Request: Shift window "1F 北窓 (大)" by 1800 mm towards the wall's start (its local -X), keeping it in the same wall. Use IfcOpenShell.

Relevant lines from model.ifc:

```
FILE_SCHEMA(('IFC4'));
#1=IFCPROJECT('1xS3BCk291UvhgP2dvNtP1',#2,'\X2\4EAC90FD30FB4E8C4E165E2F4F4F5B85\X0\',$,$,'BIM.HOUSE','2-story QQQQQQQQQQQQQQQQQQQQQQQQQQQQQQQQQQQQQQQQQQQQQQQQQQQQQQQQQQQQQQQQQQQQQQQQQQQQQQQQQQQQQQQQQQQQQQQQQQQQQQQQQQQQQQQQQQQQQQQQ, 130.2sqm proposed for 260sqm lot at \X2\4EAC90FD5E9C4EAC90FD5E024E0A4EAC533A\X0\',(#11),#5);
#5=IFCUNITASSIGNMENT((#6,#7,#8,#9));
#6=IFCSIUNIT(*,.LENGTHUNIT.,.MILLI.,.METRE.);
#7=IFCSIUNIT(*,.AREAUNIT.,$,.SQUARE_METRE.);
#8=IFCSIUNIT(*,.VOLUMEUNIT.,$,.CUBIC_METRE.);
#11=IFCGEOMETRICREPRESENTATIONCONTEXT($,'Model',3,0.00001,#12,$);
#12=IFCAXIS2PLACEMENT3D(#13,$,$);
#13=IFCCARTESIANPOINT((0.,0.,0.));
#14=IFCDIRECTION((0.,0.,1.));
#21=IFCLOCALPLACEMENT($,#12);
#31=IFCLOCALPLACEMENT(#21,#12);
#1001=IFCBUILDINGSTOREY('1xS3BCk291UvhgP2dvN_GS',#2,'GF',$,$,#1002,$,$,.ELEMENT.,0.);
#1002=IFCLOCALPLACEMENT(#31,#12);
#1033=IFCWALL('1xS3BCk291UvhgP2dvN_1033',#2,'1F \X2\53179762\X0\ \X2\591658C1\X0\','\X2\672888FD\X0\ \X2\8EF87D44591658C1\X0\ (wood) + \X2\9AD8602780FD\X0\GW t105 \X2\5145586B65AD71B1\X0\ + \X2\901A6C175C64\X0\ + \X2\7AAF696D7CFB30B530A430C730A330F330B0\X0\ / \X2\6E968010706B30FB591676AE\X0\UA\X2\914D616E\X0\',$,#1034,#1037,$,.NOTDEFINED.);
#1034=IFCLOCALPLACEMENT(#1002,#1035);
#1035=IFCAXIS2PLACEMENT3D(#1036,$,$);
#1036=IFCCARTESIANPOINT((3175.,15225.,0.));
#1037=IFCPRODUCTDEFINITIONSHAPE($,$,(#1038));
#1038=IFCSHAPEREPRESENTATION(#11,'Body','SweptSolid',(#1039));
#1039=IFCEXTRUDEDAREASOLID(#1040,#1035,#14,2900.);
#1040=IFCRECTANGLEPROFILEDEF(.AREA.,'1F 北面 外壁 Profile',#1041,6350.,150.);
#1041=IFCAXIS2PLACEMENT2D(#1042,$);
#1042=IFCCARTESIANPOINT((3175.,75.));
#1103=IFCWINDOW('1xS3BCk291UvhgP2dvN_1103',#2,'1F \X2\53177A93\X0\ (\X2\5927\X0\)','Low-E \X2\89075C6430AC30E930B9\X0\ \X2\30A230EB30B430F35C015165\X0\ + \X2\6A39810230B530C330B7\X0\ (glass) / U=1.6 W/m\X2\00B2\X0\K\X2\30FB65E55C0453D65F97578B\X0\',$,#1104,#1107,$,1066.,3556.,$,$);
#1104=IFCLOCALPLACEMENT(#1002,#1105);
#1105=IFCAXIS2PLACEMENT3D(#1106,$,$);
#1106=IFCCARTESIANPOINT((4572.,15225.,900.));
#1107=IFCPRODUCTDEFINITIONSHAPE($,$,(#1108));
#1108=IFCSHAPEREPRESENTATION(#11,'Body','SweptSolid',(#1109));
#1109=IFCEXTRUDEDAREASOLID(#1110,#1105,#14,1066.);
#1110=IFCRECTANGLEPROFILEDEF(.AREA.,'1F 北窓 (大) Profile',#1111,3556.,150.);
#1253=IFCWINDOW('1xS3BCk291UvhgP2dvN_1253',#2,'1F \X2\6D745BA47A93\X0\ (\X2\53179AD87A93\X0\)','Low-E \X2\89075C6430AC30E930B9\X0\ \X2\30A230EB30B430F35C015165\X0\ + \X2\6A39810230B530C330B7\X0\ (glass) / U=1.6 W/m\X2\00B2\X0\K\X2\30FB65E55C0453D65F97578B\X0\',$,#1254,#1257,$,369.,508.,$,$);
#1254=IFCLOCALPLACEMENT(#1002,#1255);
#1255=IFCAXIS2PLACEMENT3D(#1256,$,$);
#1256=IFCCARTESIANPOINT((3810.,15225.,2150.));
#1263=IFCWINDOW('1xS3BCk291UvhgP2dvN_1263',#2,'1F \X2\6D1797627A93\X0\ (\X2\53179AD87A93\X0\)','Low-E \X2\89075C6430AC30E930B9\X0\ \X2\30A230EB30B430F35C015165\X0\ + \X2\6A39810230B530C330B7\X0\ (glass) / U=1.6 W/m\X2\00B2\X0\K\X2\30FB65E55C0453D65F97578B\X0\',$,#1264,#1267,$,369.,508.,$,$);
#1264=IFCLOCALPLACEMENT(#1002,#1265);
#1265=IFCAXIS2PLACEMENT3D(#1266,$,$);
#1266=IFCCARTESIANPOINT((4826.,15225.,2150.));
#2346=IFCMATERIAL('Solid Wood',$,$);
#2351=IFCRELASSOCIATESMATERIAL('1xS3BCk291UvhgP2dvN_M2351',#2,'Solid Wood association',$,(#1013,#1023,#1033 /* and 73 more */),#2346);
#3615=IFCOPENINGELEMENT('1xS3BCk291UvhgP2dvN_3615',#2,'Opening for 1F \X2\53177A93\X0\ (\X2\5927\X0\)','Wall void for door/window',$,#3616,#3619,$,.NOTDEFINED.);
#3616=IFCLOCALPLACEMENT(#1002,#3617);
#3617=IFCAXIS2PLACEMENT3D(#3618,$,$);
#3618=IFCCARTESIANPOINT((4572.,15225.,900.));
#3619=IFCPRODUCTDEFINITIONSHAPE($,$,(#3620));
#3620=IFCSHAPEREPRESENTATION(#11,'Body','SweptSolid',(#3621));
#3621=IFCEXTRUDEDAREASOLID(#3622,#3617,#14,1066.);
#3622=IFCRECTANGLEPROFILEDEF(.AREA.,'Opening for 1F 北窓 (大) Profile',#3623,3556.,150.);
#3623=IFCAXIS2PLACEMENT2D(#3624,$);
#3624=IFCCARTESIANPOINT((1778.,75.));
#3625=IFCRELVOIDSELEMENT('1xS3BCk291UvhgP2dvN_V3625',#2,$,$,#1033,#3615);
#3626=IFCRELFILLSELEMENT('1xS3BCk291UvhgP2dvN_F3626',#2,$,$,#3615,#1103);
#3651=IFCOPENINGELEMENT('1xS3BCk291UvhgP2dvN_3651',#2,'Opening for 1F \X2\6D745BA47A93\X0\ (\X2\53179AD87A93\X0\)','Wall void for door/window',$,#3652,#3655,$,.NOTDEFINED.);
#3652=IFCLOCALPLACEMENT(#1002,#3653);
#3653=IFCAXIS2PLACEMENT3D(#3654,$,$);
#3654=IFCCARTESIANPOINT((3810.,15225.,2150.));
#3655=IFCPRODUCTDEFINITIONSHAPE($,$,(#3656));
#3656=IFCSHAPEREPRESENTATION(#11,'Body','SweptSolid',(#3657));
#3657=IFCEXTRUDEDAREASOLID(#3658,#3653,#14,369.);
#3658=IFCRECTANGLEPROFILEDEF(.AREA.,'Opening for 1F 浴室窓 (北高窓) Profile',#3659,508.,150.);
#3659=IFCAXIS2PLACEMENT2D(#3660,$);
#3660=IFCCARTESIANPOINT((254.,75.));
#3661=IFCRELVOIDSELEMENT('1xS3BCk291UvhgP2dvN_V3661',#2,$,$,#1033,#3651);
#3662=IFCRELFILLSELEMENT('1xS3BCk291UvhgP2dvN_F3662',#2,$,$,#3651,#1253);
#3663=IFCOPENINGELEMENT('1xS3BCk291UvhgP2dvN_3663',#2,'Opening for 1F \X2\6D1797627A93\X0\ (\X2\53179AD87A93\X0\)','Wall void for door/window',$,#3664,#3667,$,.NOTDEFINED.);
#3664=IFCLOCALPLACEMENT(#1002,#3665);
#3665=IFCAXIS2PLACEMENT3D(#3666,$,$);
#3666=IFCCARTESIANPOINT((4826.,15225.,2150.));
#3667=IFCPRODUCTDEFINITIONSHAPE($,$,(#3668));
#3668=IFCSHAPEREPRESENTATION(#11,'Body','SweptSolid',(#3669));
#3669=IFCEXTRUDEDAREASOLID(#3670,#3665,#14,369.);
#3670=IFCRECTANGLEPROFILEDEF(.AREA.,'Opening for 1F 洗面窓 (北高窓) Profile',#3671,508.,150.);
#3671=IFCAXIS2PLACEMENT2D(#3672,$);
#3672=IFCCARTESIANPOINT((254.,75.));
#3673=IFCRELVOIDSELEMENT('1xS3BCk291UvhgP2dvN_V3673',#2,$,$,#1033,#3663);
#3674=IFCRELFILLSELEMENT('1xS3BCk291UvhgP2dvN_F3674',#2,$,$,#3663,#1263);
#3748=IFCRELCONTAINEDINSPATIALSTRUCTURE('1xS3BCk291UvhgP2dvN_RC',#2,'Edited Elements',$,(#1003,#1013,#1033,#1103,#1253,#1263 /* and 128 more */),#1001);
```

```python
import ifcopenshell
import ifcopenshell.api.geometry
import ifcopenshell.util.placement
import ifcopenshell.util.unit

model = ifcopenshell.open("model.ifc")
unit_scale = ifcopenshell.util.unit.calculate_unit_scale(model)

window = model.by_guid("1xS3BCk291UvhgP2dvN_1103")
opening = window.FillsVoids[0].RelatingOpeningElement
wall = opening.VoidsElements[0].RelatingBuildingElement

wall_matrix = ifcopenshell.util.placement.get_local_placement(wall.ObjectPlacement)
shift = wall_matrix[:3, 0] * -1.8 / unit_scale
before = ifcopenshell.util.placement.get_local_placement(window.ObjectPlacement)[:3, 3].copy()

# The window is not placed relative to its opening, so move both.
for product in (opening, window):
    matrix = ifcopenshell.util.placement.get_local_placement(product.ObjectPlacement)
    matrix[:3, 3] += shift
    ifcopenshell.api.geometry.edit_object_placement(model, product=product, matrix=matrix, is_si=False)

after = ifcopenshell.util.placement.get_local_placement(window.ObjectPlacement)[:3, 3]
print("window moved by", (after - before).round(3) + 0.0)

model.write("model_v2.ifc")
```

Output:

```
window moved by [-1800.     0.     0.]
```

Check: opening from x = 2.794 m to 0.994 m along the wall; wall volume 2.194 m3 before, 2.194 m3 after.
